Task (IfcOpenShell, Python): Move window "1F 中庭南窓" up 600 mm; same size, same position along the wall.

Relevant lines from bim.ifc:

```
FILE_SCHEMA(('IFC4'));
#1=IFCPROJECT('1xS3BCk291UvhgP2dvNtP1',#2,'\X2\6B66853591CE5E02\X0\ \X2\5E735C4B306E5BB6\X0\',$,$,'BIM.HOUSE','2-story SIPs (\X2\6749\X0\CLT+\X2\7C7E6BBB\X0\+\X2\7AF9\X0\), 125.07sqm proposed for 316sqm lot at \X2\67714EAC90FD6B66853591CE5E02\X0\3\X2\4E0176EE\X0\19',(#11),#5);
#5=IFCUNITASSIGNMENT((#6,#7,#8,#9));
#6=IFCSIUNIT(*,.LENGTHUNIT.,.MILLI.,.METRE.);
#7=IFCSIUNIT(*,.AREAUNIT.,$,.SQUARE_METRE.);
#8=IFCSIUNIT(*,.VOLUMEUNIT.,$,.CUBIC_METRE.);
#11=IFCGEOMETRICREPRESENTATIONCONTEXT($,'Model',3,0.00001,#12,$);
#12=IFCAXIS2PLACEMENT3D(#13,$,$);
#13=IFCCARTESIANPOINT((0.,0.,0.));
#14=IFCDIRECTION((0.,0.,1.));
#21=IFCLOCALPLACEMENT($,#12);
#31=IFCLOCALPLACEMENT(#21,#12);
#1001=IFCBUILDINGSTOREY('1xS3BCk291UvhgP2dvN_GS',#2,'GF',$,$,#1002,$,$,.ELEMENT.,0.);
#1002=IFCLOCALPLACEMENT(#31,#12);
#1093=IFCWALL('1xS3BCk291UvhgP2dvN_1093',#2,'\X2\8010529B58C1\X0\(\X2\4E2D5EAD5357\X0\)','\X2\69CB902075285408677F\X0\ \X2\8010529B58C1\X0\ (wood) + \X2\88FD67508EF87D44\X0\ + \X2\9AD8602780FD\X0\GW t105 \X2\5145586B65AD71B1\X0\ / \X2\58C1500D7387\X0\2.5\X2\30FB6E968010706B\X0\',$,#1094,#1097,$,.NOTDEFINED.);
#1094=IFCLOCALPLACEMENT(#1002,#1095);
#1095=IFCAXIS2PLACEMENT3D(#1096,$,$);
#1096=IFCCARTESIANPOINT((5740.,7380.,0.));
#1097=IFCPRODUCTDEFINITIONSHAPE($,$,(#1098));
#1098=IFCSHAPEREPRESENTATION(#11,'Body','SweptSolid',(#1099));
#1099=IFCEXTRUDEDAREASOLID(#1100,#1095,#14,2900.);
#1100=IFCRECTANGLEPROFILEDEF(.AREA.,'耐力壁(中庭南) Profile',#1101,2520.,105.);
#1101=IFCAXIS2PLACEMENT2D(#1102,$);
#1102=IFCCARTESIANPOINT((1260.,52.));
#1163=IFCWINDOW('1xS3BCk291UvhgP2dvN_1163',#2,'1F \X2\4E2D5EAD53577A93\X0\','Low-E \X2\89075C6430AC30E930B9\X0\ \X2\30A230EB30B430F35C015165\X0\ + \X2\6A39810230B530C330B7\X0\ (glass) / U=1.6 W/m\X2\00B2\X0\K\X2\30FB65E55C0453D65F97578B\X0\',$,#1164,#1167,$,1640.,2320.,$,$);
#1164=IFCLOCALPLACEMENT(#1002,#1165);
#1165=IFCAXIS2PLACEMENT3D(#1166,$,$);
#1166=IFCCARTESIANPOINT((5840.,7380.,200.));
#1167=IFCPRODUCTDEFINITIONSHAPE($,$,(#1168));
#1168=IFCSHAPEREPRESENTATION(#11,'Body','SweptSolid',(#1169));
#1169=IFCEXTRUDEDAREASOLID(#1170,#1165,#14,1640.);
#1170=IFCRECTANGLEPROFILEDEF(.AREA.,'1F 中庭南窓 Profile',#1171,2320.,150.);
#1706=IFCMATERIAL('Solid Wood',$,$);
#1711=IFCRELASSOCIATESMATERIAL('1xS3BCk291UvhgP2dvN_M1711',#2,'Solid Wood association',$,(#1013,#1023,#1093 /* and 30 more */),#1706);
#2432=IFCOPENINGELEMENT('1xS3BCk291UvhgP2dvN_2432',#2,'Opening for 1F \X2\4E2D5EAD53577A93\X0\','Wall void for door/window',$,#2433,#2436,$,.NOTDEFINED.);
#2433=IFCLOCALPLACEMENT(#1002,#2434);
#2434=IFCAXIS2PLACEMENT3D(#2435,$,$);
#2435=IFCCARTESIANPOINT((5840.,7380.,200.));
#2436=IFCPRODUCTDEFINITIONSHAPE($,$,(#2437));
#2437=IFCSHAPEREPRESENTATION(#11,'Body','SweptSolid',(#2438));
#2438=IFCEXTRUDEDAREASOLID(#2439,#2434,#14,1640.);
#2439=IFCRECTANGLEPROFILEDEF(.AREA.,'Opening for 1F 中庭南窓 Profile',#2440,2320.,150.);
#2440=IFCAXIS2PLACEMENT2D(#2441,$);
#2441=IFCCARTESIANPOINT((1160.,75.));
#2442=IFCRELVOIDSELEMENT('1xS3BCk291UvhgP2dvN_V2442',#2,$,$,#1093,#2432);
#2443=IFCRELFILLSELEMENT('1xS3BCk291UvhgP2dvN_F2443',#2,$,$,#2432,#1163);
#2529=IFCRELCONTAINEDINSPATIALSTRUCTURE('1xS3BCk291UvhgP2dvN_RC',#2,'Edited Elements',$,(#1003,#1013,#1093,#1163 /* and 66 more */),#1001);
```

```python
import numpy as np
import ifcopenshell
import ifcopenshell.api.geometry
import ifcopenshell.util.placement
import ifcopenshell.util.unit

model = ifcopenshell.open("bim.ifc")
unit_scale = ifcopenshell.util.unit.calculate_unit_scale(model)

window = model.by_guid("1xS3BCk291UvhgP2dvN_1163")
opening = window.FillsVoids[0].RelatingOpeningElement
dz = 600.0

shift = np.array([0.0, 0.0, dz])
# The window is not placed relative to its opening, so move both.
for product in (opening, window):
    matrix = ifcopenshell.util.placement.get_local_placement(product.ObjectPlacement)
    matrix[:3, 3] += shift
    ifcopenshell.api.geometry.edit_object_placement(model, product=product, matrix=matrix, is_si=False)

print(f"moved by {dz * unit_scale:+.3f} m")

model.write("bim_rev.ifc")
```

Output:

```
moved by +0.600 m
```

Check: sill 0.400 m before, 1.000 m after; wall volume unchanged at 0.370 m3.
